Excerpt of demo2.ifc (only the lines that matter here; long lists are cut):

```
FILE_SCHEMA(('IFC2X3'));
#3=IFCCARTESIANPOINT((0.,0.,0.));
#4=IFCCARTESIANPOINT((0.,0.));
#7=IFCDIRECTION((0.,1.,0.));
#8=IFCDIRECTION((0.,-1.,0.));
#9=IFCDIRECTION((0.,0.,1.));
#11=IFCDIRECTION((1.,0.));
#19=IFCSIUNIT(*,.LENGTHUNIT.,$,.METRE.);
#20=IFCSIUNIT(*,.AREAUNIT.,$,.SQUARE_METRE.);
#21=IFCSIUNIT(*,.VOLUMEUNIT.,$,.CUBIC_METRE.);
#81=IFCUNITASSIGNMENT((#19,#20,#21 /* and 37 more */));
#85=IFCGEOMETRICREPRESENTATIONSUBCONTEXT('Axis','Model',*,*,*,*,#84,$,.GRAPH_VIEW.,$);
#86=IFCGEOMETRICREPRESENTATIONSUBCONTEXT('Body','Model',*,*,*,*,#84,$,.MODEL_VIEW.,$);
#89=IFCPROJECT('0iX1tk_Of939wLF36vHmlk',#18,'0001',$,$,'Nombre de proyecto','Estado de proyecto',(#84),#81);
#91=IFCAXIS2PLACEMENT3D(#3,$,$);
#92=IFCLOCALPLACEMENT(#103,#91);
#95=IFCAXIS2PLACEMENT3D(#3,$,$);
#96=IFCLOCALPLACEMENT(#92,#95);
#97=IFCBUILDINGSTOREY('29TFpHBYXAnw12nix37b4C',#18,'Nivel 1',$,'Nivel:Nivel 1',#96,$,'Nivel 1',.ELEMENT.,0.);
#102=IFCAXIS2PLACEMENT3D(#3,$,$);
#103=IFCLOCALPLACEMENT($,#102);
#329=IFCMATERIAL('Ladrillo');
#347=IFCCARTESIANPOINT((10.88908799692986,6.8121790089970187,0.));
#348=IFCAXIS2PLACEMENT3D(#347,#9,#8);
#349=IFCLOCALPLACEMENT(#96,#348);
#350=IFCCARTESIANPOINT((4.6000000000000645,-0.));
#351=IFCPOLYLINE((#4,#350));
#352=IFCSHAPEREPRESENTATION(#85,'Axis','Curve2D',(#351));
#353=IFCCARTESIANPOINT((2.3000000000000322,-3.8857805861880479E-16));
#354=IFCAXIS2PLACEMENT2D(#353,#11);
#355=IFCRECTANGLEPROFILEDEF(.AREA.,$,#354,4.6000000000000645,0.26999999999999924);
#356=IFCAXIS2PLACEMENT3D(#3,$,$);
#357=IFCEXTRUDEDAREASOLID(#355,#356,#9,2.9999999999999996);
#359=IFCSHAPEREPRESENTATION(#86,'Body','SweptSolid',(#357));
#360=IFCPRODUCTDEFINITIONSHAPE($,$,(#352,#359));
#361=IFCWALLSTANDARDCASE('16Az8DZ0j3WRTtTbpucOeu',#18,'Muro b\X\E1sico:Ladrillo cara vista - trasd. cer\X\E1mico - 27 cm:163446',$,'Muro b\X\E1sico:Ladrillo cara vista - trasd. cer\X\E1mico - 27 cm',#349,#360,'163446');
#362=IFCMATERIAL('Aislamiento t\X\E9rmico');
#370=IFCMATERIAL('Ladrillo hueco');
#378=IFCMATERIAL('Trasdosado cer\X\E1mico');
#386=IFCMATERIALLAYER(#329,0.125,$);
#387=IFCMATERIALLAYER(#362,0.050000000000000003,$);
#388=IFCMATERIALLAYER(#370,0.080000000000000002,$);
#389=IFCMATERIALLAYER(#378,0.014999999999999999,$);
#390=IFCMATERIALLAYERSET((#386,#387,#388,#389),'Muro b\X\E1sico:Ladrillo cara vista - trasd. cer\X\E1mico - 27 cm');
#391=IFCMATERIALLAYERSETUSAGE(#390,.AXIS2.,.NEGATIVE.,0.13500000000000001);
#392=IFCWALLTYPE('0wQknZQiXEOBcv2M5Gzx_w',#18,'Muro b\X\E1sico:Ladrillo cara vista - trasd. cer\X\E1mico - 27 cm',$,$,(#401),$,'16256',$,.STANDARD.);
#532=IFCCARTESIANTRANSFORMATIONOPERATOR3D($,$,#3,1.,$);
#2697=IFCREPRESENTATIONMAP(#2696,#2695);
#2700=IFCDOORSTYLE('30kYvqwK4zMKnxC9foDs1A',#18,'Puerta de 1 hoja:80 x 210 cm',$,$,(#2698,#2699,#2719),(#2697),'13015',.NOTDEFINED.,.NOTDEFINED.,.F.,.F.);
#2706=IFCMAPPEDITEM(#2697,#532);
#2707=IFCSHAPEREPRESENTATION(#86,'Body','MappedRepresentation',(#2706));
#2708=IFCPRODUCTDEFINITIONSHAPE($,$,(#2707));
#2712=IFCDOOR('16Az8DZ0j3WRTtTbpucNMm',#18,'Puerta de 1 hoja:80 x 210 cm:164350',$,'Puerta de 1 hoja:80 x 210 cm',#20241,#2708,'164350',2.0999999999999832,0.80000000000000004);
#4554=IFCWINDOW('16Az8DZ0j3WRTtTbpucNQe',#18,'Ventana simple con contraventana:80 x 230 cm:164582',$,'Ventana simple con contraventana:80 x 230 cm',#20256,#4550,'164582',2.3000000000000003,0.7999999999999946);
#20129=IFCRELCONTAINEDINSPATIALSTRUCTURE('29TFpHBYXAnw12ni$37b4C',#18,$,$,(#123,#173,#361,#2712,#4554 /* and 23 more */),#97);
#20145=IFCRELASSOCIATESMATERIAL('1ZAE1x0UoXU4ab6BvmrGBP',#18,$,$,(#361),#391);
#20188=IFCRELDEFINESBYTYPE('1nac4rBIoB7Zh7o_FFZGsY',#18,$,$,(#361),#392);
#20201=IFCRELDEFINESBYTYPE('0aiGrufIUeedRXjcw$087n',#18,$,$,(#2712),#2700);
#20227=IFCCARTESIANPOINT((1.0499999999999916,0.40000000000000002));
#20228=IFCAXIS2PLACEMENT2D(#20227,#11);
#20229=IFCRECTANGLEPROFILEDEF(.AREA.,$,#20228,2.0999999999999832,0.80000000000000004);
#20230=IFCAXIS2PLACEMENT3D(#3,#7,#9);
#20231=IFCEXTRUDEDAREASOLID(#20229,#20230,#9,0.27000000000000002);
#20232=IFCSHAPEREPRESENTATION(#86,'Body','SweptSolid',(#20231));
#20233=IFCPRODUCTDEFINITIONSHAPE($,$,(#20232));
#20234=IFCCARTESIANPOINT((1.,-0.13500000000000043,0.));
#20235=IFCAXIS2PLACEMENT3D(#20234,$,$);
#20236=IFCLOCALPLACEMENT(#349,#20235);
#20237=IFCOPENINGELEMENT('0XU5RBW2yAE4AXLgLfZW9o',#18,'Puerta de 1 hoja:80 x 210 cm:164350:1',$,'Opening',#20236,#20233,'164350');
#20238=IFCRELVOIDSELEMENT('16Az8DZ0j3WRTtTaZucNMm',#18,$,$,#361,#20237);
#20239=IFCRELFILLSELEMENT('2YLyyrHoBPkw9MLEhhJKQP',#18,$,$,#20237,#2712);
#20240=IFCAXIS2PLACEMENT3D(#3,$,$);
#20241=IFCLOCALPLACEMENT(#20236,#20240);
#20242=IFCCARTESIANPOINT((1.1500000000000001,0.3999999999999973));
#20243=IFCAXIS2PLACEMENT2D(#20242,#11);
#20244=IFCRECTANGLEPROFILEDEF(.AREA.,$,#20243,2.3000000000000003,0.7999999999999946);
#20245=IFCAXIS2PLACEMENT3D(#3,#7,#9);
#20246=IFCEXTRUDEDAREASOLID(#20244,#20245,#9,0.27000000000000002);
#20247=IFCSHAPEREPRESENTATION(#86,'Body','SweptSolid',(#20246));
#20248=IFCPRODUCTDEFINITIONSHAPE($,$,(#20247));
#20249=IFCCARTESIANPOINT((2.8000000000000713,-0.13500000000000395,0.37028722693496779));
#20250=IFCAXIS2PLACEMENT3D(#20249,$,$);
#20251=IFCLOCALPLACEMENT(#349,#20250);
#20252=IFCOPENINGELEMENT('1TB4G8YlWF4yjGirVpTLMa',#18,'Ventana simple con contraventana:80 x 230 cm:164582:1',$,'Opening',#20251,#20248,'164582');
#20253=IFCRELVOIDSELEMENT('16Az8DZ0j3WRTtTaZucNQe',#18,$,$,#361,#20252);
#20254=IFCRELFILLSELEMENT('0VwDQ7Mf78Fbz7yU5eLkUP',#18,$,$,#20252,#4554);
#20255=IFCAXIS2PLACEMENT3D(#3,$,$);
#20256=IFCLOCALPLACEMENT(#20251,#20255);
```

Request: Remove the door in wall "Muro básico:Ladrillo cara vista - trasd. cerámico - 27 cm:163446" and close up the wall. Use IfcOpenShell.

```python
import ifcopenshell
import ifcopenshell.api.feature
import ifcopenshell.api.root
import ifcopenshell.geom
import ifcopenshell.util.shape

model = ifcopenshell.open("demo2.ifc")
settings = ifcopenshell.geom.settings()


def volume(element):
    """Net volume in cubic metres, openings subtracted."""
    shape = ifcopenshell.geom.create_shape(settings, element)
    return ifcopenshell.util.shape.get_volume(shape.geometry)


door = model.by_guid("16Az8DZ0j3WRTtTbpucNMm")
opening = door.FillsVoids[0].RelatingOpeningElement
wall = opening.VoidsElements[0].RelatingBuildingElement
before = volume(wall)

ifcopenshell.api.root.remove_product(model, product=door)
ifcopenshell.api.feature.remove_feature(model, feature=opening)

after = volume(wall)

print(f"wall volume {before:.3f} -> {after:.3f} m3")

model.write("demo2-out.ifc")
```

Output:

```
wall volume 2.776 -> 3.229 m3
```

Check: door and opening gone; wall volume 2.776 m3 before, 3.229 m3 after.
